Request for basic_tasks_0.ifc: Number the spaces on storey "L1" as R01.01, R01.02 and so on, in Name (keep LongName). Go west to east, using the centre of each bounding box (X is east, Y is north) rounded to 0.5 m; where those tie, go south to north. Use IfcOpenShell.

First a look at what the model holds.

```python
import ifcopenshell
import ifcopenshell.util.element
import ifcopenshell.util.placement

model = ifcopenshell.open("basic_tasks_0.ifc")
print(model.schema)
storey = next(s for s in model.by_type("IfcBuildingStorey") if s.Name == "L1")
spaces = [e for e in ifcopenshell.util.element.get_decomposition(storey) if e.is_a("IfcSpace")]
for e in sorted(spaces, key=lambda e: e.id()):
    origin = ifcopenshell.util.placement.get_local_placement(e.ObjectPlacement)[:3, 3]
    print(e.id(), e.Name, e.LongName, origin.round(2) + 0.0, sep=" | ")
```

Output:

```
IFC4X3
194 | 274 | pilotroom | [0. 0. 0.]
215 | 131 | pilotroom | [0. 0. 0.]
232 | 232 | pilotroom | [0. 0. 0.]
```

```python
import ifcopenshell
import ifcopenshell.geom
import ifcopenshell.util.element
import ifcopenshell.util.shape

model = ifcopenshell.open("basic_tasks_0.ifc")
settings = ifcopenshell.geom.settings()
settings.set("use-world-coords", True)


def centre(element):
    shape = ifcopenshell.geom.create_shape(settings, element)
    return ifcopenshell.util.shape.get_bbox_centroid(shape.geometry)


storey = next(s for s in model.by_type("IfcBuildingStorey") if s.Name == "L1")
spaces = [e for e in ifcopenshell.util.element.get_decomposition(storey) if e.is_a("IfcSpace")]

# Insertion points can sit at a corner or the storey origin, so sort by the geometry (in metres).
centres = {e: centre(e) for e in spaces}
spaces.sort(key=lambda e: (round(centres[e][0] / 0.5), centres[e][1]))

for i, e in enumerate(spaces, start=1):
    number = f"R01.{i:02d}"
    e.Name = number
    print(e.id(), number)

model.write("basic_tasks_0_edited.ifc")
```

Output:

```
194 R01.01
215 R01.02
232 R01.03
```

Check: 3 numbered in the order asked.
